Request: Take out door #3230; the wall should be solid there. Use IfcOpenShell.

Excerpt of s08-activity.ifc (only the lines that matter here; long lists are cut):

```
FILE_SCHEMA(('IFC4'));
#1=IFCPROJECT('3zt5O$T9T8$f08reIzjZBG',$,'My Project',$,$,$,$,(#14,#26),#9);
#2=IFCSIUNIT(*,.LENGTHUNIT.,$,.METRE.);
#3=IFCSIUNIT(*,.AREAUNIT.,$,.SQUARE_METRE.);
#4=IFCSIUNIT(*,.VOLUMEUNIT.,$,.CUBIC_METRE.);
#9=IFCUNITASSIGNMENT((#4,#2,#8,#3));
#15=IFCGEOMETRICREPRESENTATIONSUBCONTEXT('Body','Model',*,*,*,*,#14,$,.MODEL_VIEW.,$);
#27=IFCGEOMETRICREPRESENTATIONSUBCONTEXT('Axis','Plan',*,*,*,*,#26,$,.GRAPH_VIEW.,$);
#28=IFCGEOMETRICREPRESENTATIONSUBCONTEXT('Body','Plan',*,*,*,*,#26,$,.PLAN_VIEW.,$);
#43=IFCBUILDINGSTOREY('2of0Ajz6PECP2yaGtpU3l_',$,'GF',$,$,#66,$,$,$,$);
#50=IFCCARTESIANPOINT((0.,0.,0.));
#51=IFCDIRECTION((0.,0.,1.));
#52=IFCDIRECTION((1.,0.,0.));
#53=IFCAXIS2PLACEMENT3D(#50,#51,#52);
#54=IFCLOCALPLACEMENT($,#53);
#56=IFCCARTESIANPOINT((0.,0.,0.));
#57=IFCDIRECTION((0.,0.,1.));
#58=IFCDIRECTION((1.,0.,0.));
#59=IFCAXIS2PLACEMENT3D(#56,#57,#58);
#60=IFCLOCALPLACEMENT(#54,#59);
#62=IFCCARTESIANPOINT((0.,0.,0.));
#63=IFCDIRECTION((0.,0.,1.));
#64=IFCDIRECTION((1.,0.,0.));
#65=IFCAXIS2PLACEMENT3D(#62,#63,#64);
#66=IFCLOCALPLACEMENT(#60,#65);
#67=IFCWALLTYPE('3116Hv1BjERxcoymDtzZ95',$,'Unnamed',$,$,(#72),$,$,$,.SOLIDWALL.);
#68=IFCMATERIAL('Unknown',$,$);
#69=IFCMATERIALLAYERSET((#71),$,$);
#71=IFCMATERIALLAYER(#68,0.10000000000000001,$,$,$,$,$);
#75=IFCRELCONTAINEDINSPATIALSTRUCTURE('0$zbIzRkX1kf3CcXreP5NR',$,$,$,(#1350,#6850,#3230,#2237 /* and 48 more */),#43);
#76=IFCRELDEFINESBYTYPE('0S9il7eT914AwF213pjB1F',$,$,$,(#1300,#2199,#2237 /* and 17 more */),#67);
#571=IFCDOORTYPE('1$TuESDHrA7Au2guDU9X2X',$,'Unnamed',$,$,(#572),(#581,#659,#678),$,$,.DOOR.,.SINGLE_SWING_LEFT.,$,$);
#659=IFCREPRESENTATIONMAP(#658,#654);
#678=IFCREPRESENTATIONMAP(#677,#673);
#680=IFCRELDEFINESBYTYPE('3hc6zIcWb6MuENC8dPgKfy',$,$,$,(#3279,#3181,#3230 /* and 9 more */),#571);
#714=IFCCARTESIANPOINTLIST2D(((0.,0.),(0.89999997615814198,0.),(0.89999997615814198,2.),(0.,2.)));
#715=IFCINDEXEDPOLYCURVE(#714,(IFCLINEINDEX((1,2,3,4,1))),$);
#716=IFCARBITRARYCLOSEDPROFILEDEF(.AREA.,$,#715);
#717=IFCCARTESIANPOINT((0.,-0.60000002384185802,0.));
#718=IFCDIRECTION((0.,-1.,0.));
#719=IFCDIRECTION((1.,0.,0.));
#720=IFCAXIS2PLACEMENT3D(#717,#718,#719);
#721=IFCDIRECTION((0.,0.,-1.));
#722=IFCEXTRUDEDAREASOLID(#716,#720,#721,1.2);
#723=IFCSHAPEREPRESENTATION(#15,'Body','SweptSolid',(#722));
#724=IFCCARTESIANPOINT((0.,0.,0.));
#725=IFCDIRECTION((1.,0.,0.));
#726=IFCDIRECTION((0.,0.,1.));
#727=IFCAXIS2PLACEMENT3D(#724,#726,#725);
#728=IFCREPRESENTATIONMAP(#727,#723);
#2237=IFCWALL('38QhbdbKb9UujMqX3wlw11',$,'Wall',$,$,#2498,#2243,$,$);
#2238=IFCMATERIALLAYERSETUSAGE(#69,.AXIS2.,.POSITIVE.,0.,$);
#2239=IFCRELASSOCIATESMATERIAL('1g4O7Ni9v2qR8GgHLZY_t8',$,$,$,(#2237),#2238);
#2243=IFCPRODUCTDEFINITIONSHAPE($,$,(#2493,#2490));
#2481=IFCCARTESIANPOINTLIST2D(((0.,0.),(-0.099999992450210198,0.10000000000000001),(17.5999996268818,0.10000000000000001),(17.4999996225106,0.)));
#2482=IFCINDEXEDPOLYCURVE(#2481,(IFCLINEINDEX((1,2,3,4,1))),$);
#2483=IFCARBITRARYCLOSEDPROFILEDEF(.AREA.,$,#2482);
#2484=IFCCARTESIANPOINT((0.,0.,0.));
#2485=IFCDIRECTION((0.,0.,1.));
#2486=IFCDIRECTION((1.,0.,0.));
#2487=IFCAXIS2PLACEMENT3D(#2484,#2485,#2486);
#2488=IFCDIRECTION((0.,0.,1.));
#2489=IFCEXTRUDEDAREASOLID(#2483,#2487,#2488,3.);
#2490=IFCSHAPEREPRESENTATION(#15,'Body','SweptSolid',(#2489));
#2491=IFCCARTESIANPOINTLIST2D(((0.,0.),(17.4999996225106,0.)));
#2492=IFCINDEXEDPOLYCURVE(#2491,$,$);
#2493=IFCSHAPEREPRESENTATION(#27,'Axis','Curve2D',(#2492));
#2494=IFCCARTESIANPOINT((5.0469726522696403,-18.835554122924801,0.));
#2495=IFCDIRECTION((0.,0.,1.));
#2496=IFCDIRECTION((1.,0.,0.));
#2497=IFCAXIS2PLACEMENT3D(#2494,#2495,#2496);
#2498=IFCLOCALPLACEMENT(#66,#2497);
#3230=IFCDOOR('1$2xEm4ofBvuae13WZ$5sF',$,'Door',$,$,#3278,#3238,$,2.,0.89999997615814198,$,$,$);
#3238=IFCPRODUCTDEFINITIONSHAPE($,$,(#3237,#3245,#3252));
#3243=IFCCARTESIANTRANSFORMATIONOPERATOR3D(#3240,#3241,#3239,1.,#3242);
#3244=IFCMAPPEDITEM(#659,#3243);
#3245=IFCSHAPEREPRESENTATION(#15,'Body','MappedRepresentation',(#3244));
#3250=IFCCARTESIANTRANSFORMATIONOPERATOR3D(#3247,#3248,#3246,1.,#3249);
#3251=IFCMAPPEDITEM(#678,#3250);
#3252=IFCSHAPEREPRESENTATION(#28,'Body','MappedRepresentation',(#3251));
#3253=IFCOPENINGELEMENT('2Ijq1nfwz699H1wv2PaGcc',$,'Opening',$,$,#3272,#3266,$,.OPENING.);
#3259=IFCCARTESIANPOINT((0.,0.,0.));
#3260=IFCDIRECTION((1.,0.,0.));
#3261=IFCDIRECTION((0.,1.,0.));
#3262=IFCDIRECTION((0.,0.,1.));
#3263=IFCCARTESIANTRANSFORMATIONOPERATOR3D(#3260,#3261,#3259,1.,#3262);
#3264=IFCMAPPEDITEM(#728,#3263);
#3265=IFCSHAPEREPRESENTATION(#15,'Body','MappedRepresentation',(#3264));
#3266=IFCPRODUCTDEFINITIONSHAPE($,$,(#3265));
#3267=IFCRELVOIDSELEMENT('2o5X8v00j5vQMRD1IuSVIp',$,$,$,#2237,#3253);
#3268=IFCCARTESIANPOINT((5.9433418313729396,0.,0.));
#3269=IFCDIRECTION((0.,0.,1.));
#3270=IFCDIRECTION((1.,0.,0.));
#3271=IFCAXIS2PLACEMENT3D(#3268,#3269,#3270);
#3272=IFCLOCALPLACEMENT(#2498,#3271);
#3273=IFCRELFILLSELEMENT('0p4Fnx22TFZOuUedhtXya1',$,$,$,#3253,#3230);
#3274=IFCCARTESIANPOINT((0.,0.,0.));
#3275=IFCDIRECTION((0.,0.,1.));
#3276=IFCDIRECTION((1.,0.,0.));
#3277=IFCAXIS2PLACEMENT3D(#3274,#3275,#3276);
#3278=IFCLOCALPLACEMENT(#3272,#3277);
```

```python
import ifcopenshell
import ifcopenshell.api.feature
import ifcopenshell.api.root
import ifcopenshell.geom
import ifcopenshell.util.shape

model = ifcopenshell.open("s08-activity.ifc")
settings = ifcopenshell.geom.settings()


def volume(element):
    """Net volume in cubic metres, openings subtracted."""
    shape = ifcopenshell.geom.create_shape(settings, element)
    return ifcopenshell.util.shape.get_volume(shape.geometry)


door = model.by_guid("1$2xEm4ofBvuae13WZ$5sF")
opening = door.FillsVoids[0].RelatingOpeningElement
wall = opening.VoidsElements[0].RelatingBuildingElement
before = volume(wall)

ifcopenshell.api.root.remove_product(model, product=door)
ifcopenshell.api.feature.remove_feature(model, feature=opening)

after = volume(wall)

print(f"wall volume {before:.3f} -> {after:.3f} m3")

model.write("s08-activity_rev.ifc")
```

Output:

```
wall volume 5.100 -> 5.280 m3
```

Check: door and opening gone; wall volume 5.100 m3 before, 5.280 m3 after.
